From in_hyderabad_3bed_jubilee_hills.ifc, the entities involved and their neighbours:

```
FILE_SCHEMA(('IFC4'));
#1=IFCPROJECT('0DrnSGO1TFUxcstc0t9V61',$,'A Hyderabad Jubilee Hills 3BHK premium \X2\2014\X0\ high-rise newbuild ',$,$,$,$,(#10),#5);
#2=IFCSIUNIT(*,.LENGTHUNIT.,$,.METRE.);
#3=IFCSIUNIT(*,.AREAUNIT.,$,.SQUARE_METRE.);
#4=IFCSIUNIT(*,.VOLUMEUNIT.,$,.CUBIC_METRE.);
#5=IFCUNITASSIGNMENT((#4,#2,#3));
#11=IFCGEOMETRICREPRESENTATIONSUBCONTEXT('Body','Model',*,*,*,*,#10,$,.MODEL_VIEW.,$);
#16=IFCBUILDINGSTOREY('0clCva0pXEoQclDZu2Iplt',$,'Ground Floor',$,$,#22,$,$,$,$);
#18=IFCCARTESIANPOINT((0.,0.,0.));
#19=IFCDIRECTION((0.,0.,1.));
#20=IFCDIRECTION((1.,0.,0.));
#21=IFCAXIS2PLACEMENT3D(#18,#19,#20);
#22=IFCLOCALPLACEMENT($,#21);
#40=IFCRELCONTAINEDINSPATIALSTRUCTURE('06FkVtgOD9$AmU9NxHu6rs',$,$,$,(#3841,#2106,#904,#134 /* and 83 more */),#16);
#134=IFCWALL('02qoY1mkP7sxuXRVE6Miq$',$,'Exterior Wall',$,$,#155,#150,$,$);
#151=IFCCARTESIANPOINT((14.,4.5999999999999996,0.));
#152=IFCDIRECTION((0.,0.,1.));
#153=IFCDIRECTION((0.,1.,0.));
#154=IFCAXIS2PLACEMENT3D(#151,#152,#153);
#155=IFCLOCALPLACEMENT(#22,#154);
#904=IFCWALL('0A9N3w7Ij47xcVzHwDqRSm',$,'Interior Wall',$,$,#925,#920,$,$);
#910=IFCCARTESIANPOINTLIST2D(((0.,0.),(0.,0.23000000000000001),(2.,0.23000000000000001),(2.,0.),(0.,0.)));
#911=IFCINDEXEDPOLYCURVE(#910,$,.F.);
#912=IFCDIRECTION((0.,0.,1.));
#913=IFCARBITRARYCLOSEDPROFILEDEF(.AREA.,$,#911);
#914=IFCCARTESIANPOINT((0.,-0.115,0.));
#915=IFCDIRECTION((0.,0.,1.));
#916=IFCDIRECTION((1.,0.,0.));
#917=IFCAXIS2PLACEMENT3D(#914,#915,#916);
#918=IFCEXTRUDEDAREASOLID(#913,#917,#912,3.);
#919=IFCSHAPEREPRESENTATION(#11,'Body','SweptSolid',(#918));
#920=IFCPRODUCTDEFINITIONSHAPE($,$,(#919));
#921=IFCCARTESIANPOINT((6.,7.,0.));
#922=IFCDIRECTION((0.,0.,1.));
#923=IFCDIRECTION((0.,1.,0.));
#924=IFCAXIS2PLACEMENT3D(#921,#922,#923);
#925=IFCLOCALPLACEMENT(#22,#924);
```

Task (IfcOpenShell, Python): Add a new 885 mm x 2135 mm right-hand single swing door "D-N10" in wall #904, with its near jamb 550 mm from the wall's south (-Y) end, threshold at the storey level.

```python
import numpy as np
import ifcopenshell
import ifcopenshell.api.feature
import ifcopenshell.api.geometry
import ifcopenshell.api.root
import ifcopenshell.api.spatial
import ifcopenshell.geom
import ifcopenshell.util.element
import ifcopenshell.util.placement
import ifcopenshell.util.representation
import ifcopenshell.util.shape
import ifcopenshell.util.unit

model = ifcopenshell.open("in_hyderabad_3bed_jubilee_hills.ifc")
unit_scale = ifcopenshell.util.unit.calculate_unit_scale(model)
settings = ifcopenshell.geom.settings()


def volume(element):
    """Net volume in cubic metres, openings subtracted."""
    shape = ifcopenshell.geom.create_shape(settings, element)
    return ifcopenshell.util.shape.get_volume(shape.geometry)


wall = model.by_guid("0A9N3w7Ij47xcVzHwDqRSm")
storey = ifcopenshell.util.element.get_container(wall, ifc_class="IfcBuildingStorey")
context = ifcopenshell.util.representation.get_context(model, "Model", "Body", "MODEL_VIEW")
before = volume(wall)

width, height, from_end, sill = 0.885, 2.135, 0.55, 0.0  # metres

# The wall runs along its own X axis, and the end named is its -X end.
wall_shape = ifcopenshell.geom.create_shape(settings, wall)
x, y, z = ifcopenshell.util.shape.get_vertices(wall_shape.geometry).T
start = x.min() + from_end
face, thickness = float(y.min()), float(y.max() - y.min())
wall_matrix = ifcopenshell.util.placement.get_local_placement(wall.ObjectPlacement)
level = ifcopenshell.util.placement.get_local_placement(storey.ObjectPlacement)[2, 3]


def in_wall(x, y):
    """Placement at x, y metres in the wall's axes, at sill height."""
    matrix = wall_matrix.copy()
    matrix[:, 3] = wall_matrix @ np.array([x / unit_scale, y / unit_scale, 0.0, 1.0])
    matrix[2, 3] = level + sill / unit_scale
    return matrix


# Opening: a box that overshoots both wall faces by 50 mm.
opening = ifcopenshell.api.root.create_entity(model, ifc_class="IfcOpeningElement", predefined_type="OPENING")
box = ifcopenshell.api.geometry.add_wall_representation(
    model, context=context, length=width, height=height, thickness=thickness + 0.1
)
ifcopenshell.api.geometry.assign_representation(model, product=opening, representation=box)
ifcopenshell.api.geometry.edit_object_placement(model, product=opening, matrix=in_wall(start, face - 0.05), is_si=False)
ifcopenshell.api.feature.add_feature(model, feature=opening, element=wall)

door = ifcopenshell.api.root.create_entity(model, ifc_class="IfcDoor", name="D-N10", predefined_type="DOOR")
door.OverallWidth, door.OverallHeight = width / unit_scale, height / unit_scale
door.OperationType = "SINGLE_SWING_RIGHT"
body = ifcopenshell.api.geometry.add_door_representation(
    model,
    context=context,
    overall_width=door.OverallWidth,
    overall_height=door.OverallHeight,
    operation_type="SINGLE_SWING_RIGHT",
    lining_properties={"LiningDepth": thickness / unit_scale, "ThresholdDepth": thickness / unit_scale},
)
ifcopenshell.api.geometry.assign_representation(model, product=door, representation=body)
ifcopenshell.api.spatial.assign_container(model, products=[door], relating_structure=storey)
ifcopenshell.api.feature.add_filling(model, opening=opening, element=door)

# The lining spans the wall, so the door starts at the wall face.
ifcopenshell.api.geometry.edit_object_placement(model, product=door, matrix=in_wall(start, face), is_si=False)

after = volume(wall)

print(f"wall volume {before:.3f} -> {after:.3f} m3")

model.write("in_hyderabad_3bed_jubilee_hills_updated.ifc")
```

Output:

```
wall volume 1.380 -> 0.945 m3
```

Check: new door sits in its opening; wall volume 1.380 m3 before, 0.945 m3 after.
